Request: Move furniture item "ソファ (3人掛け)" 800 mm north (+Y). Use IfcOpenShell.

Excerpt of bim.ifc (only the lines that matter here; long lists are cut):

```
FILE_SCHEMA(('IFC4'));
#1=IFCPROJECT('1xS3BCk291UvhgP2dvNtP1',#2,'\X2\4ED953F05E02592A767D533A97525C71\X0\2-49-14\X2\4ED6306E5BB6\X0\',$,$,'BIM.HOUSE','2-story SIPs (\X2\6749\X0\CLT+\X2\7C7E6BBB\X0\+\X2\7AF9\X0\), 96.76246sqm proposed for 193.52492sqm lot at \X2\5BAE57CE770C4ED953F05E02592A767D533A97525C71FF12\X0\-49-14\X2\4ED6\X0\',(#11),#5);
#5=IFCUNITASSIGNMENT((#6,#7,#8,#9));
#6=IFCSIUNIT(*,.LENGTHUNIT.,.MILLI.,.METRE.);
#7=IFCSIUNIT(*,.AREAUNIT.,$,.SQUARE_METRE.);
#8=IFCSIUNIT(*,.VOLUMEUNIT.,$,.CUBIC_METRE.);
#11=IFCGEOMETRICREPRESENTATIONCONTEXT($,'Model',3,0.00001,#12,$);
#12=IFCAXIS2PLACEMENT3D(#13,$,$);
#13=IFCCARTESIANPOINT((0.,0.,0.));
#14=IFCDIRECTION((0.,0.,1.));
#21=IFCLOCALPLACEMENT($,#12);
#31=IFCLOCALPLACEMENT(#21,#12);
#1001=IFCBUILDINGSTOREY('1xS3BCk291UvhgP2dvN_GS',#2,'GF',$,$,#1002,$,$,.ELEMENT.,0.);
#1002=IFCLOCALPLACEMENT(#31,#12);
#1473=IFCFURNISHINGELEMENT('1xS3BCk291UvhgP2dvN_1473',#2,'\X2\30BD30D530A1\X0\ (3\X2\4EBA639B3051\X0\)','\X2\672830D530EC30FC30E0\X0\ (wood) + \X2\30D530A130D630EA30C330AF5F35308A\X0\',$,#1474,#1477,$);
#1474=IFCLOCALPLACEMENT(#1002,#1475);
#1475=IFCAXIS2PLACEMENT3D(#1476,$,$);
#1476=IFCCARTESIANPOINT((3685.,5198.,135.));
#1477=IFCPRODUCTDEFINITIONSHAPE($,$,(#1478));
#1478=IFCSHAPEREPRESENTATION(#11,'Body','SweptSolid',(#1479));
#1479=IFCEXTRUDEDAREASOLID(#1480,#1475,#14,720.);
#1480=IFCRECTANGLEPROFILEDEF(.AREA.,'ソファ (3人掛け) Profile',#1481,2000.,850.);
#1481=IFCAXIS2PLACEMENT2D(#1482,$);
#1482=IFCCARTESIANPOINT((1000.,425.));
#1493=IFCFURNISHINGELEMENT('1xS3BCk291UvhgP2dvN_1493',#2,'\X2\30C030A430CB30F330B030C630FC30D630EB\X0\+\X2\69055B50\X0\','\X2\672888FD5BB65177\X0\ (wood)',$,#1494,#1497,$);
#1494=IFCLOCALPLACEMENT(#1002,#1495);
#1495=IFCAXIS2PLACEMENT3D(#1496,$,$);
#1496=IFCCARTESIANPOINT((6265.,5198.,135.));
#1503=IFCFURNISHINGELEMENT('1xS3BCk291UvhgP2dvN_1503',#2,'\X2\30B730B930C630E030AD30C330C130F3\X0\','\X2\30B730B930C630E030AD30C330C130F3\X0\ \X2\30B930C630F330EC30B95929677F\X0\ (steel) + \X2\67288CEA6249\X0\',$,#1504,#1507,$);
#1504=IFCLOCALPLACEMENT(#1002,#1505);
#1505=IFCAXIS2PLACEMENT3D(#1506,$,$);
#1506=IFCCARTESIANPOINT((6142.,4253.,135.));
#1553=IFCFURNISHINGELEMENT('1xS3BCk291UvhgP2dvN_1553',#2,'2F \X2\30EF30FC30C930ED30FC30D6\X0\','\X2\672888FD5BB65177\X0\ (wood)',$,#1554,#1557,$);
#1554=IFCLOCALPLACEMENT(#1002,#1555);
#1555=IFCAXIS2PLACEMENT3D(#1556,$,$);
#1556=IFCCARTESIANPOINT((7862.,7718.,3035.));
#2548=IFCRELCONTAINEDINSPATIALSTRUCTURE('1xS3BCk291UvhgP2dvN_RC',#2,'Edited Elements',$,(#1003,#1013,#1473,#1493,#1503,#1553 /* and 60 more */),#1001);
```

```python
import ifcopenshell
import ifcopenshell.api.geometry
import ifcopenshell.util.placement
import ifcopenshell.util.unit

model = ifcopenshell.open("bim.ifc")
unit_scale = ifcopenshell.util.unit.calculate_unit_scale(model)

item = model.by_guid("1xS3BCk291UvhgP2dvN_1473")
matrix = ifcopenshell.util.placement.get_local_placement(item.ObjectPlacement)
matrix[1, 3] += 0.8 / unit_scale
ifcopenshell.api.geometry.edit_object_placement(model, product=item, matrix=matrix, is_si=False)

print(ifcopenshell.util.placement.get_local_placement(item.ObjectPlacement).round(3) + 0.0)

model.write("bim_updated.ifc")
```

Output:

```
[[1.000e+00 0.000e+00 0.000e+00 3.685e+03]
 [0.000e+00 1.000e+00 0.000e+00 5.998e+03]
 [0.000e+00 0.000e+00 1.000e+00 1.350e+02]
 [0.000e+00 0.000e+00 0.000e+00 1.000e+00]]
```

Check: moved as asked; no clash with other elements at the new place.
